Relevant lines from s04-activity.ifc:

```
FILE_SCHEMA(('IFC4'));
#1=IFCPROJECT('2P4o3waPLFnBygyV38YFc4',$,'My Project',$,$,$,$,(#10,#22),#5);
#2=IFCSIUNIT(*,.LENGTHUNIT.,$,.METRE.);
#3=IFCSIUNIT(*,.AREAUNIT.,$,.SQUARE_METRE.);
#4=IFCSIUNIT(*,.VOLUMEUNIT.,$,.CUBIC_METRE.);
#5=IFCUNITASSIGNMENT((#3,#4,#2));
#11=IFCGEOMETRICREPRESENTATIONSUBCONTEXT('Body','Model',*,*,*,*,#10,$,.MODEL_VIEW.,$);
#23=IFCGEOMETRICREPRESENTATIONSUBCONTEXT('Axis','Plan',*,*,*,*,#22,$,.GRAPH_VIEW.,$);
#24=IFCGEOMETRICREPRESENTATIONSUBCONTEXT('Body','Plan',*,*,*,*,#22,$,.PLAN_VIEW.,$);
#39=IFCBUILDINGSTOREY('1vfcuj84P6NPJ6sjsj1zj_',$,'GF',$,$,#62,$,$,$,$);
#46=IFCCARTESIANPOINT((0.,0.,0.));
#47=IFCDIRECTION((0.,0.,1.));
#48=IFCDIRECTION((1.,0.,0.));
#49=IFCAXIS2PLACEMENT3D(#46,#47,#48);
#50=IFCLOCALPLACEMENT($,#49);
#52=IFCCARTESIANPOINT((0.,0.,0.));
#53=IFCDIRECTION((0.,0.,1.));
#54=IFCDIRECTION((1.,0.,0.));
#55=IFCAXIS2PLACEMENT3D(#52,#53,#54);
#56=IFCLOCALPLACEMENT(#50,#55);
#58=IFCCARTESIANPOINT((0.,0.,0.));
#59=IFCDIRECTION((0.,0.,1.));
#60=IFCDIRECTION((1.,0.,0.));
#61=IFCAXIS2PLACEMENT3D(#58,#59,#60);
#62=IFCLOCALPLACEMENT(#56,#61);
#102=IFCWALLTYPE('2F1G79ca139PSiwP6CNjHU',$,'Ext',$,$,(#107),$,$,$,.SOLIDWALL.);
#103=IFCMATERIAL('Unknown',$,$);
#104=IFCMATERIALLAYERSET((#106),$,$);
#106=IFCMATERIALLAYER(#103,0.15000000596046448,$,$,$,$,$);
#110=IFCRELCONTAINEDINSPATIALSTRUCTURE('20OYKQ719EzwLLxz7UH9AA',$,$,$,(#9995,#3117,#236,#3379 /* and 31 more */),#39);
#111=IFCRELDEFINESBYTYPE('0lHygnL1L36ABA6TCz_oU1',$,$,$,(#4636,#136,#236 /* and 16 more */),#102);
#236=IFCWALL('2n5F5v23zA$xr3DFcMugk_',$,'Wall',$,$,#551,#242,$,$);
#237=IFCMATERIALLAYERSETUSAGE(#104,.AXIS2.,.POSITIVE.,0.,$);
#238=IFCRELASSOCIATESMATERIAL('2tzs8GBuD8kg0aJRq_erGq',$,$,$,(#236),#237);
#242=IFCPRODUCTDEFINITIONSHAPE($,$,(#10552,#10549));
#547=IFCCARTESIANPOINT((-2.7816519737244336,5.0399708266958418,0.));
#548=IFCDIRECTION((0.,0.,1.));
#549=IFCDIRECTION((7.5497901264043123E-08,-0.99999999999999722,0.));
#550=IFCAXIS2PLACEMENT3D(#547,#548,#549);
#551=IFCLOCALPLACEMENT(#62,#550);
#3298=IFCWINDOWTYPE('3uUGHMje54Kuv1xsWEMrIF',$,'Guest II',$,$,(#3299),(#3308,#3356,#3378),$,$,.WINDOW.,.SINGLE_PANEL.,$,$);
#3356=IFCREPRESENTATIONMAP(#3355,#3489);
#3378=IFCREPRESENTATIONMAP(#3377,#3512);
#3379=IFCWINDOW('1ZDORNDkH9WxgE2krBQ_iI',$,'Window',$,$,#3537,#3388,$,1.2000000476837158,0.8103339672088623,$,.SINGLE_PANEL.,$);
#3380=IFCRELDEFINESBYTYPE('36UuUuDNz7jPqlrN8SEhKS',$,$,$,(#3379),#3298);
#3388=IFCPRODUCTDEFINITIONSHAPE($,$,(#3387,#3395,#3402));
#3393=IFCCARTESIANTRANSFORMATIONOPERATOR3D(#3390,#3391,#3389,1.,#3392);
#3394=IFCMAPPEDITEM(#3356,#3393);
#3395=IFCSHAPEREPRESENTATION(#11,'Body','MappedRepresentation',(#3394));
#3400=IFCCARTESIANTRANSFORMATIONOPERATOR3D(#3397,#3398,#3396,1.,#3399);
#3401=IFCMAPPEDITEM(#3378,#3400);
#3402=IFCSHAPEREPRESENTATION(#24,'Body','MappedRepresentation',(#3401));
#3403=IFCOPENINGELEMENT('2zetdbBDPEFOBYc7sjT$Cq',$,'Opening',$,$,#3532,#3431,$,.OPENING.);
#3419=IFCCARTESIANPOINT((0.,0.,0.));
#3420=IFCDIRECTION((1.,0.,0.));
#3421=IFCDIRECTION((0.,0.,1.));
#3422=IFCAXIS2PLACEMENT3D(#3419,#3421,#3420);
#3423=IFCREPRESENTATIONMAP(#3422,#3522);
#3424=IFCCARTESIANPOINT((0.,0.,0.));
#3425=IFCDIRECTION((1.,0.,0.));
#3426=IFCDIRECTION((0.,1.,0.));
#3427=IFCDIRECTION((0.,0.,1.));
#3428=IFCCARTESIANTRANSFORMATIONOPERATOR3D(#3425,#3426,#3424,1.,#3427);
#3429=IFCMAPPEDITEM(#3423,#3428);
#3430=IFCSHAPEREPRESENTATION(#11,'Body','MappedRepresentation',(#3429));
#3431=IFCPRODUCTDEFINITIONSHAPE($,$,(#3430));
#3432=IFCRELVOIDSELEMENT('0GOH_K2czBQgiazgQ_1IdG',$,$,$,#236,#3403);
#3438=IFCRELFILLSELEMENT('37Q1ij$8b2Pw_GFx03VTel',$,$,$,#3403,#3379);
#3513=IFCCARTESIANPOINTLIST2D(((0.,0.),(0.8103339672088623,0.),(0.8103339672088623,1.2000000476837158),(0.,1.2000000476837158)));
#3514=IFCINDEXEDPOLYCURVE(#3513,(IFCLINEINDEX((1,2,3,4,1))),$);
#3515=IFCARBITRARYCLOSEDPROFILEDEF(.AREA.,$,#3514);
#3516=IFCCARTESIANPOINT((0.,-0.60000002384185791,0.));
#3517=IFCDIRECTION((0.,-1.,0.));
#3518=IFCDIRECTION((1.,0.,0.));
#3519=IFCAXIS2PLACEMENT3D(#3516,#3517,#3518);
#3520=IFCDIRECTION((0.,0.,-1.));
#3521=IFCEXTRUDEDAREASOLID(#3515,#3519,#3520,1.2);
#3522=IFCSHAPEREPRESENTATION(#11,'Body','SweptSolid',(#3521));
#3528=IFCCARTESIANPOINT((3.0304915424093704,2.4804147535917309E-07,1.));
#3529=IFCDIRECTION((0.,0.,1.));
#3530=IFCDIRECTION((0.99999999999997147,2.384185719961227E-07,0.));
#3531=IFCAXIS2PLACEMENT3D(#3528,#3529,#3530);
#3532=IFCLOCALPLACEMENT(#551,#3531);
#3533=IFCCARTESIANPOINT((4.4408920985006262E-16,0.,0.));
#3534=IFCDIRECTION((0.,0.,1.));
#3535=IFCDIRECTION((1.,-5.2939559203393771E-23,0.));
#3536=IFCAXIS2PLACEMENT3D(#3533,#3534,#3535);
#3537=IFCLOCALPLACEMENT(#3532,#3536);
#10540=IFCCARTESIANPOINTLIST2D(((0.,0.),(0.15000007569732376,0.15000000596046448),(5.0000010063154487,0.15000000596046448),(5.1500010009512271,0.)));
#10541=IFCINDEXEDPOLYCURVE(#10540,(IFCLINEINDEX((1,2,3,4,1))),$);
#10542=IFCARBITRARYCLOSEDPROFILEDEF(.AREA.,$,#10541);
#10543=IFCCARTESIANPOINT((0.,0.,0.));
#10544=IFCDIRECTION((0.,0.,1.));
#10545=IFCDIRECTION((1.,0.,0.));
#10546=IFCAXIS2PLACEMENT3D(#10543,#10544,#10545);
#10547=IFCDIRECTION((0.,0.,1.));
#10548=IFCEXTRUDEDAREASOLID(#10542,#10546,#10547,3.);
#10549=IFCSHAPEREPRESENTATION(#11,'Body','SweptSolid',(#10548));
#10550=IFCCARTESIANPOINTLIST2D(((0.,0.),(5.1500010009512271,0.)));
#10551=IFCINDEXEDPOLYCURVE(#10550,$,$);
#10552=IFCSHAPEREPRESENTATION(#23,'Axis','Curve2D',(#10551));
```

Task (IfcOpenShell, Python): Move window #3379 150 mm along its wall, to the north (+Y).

```python
import ifcopenshell
import ifcopenshell.api.geometry
import ifcopenshell.util.placement
import ifcopenshell.util.unit

model = ifcopenshell.open("s04-activity.ifc")
unit_scale = ifcopenshell.util.unit.calculate_unit_scale(model)

window = model.by_id(3379)
opening = window.FillsVoids[0].RelatingOpeningElement
wall = opening.VoidsElements[0].RelatingBuildingElement

wall_matrix = ifcopenshell.util.placement.get_local_placement(wall.ObjectPlacement)
shift = wall_matrix[:3, 0] * -0.15 / unit_scale
before = ifcopenshell.util.placement.get_local_placement(window.ObjectPlacement)[:3, 3].copy()

# The window is placed relative to its opening, so it follows when the opening moves.
matrix = ifcopenshell.util.placement.get_local_placement(opening.ObjectPlacement)
matrix[:3, 3] += shift
ifcopenshell.api.geometry.edit_object_placement(
    model, product=opening, matrix=matrix, is_si=False, should_transform_children=True
)

after = ifcopenshell.util.placement.get_local_placement(window.ObjectPlacement)[:3, 3]
print("window moved by", (after - before).round(3) + 0.0)

model.write("s04-activity-out.ifc")
```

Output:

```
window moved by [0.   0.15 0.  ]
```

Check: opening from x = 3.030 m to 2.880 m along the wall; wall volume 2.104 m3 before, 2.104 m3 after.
